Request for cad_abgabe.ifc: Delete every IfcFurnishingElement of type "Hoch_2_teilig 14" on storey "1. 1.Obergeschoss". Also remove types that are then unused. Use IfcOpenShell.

First a look at what the model holds.

```python
import ifcopenshell
import ifcopenshell.util.element

model = ifcopenshell.open("cad_abgabe.ifc")
print(model.schema)
storey = next(s for s in model.by_type("IfcBuildingStorey") if s.Name == "1. 1.Obergeschoss")
furniture = [e for e in ifcopenshell.util.element.get_decomposition(storey) if e.is_a("IfcFurnishingElement")]
seen = {}
for e in furniture:
    element_type = ifcopenshell.util.element.get_type(e)
    name = element_type.Name if element_type not in (None, e) else None
    seen[name] = seen.get(name, 0) + 1
for name, count in sorted(seen.items(), key=str):
    print(count, "x", name)
```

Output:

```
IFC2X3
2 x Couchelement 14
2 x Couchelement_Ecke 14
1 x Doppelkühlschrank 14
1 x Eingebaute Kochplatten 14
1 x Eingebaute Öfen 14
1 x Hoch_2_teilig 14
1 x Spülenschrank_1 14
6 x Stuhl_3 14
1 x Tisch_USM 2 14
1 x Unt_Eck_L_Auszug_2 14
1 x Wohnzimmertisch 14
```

```python
import ifcopenshell
import ifcopenshell.api.root
import ifcopenshell.util.element

model = ifcopenshell.open("cad_abgabe.ifc")

storey = next(s for s in model.by_type("IfcBuildingStorey") if s.Name == "1. 1.Obergeschoss")
furniture = [e for e in ifcopenshell.util.element.get_decomposition(storey) if e.is_a("IfcFurnishingElement")]
targets = [e for e in furniture if (t := ifcopenshell.util.element.get_type(e)) not in (None, e) and t.Name == "Hoch_2_teilig 14"]
types = {ifcopenshell.util.element.get_type(e) for e in targets} - {None, *targets}

for e in targets:
    ifcopenshell.api.root.remove_product(model, product=e)
print(len(targets), "removed")

unused = [t for t in types if not ifcopenshell.util.element.get_types(t)]
for t in unused:
    ifcopenshell.api.root.remove_product(model, product=t)
print(len(unused), "unused types removed")

model.write("cad_abgabe_edited.ifc")
```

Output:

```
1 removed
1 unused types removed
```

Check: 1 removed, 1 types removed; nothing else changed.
